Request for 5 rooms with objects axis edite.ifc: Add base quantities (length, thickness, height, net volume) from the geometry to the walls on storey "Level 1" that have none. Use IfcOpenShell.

First a look at what the model holds.

```python
import ifcopenshell
import ifcopenshell.util.element
import ifcopenshell.util.unit

model = ifcopenshell.open("5 rooms with objects axis edite.ifc")
print(model.schema)
for unit_type in ("LENGTHUNIT", "AREAUNIT", "VOLUMEUNIT"):
    print(unit_type, ifcopenshell.util.unit.calculate_unit_scale(model, unit_type))
storey = next(s for s in model.by_type("IfcBuildingStorey") if s.Name == "Level 1")
walls = [e for e in ifcopenshell.util.element.get_decomposition(storey) if e.is_a("IfcWall")]
for e in sorted(walls, key=lambda e: e.id()):
    print(e.id(), e.is_a(), e.Name, list(ifcopenshell.util.element.get_psets(e, qtos_only=True)), sep=" | ")
```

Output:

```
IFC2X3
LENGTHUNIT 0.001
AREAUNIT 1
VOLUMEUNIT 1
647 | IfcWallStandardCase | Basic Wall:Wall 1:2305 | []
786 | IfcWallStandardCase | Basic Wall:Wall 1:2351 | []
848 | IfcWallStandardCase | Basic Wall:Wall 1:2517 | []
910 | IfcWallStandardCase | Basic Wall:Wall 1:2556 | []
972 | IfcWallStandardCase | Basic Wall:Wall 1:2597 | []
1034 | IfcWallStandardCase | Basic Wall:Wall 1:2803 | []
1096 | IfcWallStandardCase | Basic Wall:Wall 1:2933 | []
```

```python
import ifcopenshell
import ifcopenshell.api.pset
import ifcopenshell.geom
import ifcopenshell.util.element
import ifcopenshell.util.shape
import ifcopenshell.util.unit

model = ifcopenshell.open("5 rooms with objects axis edite.ifc")
unit_scale = ifcopenshell.util.unit.calculate_unit_scale(model)
volume_scale = ifcopenshell.util.unit.calculate_unit_scale(model, "VOLUMEUNIT")
settings = ifcopenshell.geom.settings()

storey = next(s for s in model.by_type("IfcBuildingStorey") if s.Name == "Level 1")
walls = [e for e in ifcopenshell.util.element.get_decomposition(storey) if e.is_a("IfcWall")]

for e in sorted(walls, key=lambda e: e.id()):
    if ifcopenshell.util.element.get_psets(e, qtos_only=True, should_inherit=False):
        continue
    # Geometry comes back in metres, in the element's own axes.
    shape = ifcopenshell.geom.create_shape(settings, e)
    values = {
        "Length": ifcopenshell.util.shape.get_x(shape.geometry) / unit_scale,
        "Width": ifcopenshell.util.shape.get_y(shape.geometry) / unit_scale,
        "Height": ifcopenshell.util.shape.get_z(shape.geometry) / unit_scale,
        "NetVolume": ifcopenshell.util.shape.get_volume(shape.geometry) / volume_scale,
    }
    qto = ifcopenshell.api.pset.add_qto(model, product=e, name="BaseQuantities")
    ifcopenshell.api.pset.edit_qto(model, qto=qto, properties=values)
    print(e.id(), {k: round(v, 3) for k, v in values.items()})

model.write("5 rooms with objects axis edite_rev.ifc")
```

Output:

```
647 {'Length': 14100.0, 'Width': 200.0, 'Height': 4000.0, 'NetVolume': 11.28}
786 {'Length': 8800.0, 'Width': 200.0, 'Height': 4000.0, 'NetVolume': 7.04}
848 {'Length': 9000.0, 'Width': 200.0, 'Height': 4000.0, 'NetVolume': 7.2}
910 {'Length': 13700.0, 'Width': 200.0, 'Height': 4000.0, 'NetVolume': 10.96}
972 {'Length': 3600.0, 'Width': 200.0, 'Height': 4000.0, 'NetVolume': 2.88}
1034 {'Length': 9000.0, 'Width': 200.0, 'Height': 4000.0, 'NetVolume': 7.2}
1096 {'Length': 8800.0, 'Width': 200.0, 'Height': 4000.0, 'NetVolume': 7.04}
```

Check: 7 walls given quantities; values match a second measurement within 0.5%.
